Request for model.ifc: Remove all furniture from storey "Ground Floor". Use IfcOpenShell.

First a look at what the model holds.

```python
import ifcopenshell
import ifcopenshell.util.element

model = ifcopenshell.open("model.ifc")
print(model.schema)
storey = next(s for s in model.by_type("IfcBuildingStorey") if s.Name == "Ground Floor")
furniture = [e for e in ifcopenshell.util.element.get_decomposition(storey) if e.is_a("IfcFurnishingElement")]
seen = {}
for e in furniture:
    element_type = ifcopenshell.util.element.get_type(e)
    name = element_type.Name if element_type not in (None, e) else None
    seen[name] = seen.get(name, 0) + 1
for name, count in sorted(seen.items(), key=str):
    print(count, "x", name)
```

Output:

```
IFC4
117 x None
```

```python
import ifcopenshell
import ifcopenshell.api.root
import ifcopenshell.util.element

model = ifcopenshell.open("model.ifc")

storey = next(s for s in model.by_type("IfcBuildingStorey") if s.Name == "Ground Floor")
furniture = [e for e in ifcopenshell.util.element.get_decomposition(storey) if e.is_a("IfcFurnishingElement")]

for e in furniture:
    ifcopenshell.api.root.remove_product(model, product=e)
print(len(furniture), "removed")

model.write("model_edited.ifc")
```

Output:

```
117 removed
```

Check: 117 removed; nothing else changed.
